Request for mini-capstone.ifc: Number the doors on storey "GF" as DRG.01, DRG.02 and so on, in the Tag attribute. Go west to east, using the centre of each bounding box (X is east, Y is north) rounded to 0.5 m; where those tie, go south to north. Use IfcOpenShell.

First a look at what the model holds.

```python
import ifcopenshell
import ifcopenshell.util.element
import ifcopenshell.util.placement

model = ifcopenshell.open("mini-capstone.ifc")
print(model.schema)
storey = next(s for s in model.by_type("IfcBuildingStorey") if s.Name == "GF")
doors = [e for e in ifcopenshell.util.element.get_decomposition(storey) if e.is_a("IfcDoor")]
for e in sorted(doors, key=lambda e: e.id()):
    origin = ifcopenshell.util.placement.get_local_placement(e.ObjectPlacement)[:3, 3]
    print(e.id(), e.Tag, e.Name, origin.round(2) + 0.0, sep=" | ")
```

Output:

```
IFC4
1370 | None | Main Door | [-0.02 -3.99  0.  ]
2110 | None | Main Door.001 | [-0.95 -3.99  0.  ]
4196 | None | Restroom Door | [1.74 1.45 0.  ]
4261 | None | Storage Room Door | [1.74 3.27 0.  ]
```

```python
import ifcopenshell
import ifcopenshell.geom
import ifcopenshell.util.element
import ifcopenshell.util.shape

model = ifcopenshell.open("mini-capstone.ifc")
settings = ifcopenshell.geom.settings()
settings.set("use-world-coords", True)


def centre(element):
    shape = ifcopenshell.geom.create_shape(settings, element)
    return ifcopenshell.util.shape.get_bbox_centroid(shape.geometry)


storey = next(s for s in model.by_type("IfcBuildingStorey") if s.Name == "GF")
doors = [e for e in ifcopenshell.util.element.get_decomposition(storey) if e.is_a("IfcDoor")]

# Insertion points can sit at a corner or the storey origin, so sort by the geometry (in metres).
centres = {e: centre(e) for e in doors}
doors.sort(key=lambda e: (round(centres[e][0] / 0.5), centres[e][1]))

for i, e in enumerate(doors, start=1):
    number = f"DRG.{i:02d}"
    e.Tag = number
    print(e.id(), number)

model.write("mini-capstone-out.ifc")
```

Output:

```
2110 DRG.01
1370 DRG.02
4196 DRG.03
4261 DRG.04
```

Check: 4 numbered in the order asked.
